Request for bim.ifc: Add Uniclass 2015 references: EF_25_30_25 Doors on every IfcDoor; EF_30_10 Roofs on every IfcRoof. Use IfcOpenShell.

First a look at what the model holds.

```python
import ifcopenshell

model = ifcopenshell.open("bim.ifc")
print(model.schema)
print("classifications:", [c.Name for c in model.by_type("IfcClassification")])
for ifc_class in ("IfcDoor", "IfcRoof", "IfcStair", "IfcWall", "IfcWindow"):
    print(ifc_class, len(model.by_type(ifc_class)))
```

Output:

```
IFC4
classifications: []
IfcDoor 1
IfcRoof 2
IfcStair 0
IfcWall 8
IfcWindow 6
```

```python
import ifcopenshell
import ifcopenshell.api.classification

model = ifcopenshell.open("bim.ifc")

system = ifcopenshell.api.classification.add_classification(model, classification="Uniclass 2015")

codes = {
    "IfcDoor": ("EF_25_30_25", "Doors"),
    "IfcRoof": ("EF_30_10", "Roofs"),
}
for ifc_class, (code, name) in codes.items():
    products = model.by_type(ifc_class)
    ifcopenshell.api.classification.add_reference(
        model, products=products, classification=system, identification=code, name=name
    )
    print(code, len(products))

model.write("bim_rev.ifc")
```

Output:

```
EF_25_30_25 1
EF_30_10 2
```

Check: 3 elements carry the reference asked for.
